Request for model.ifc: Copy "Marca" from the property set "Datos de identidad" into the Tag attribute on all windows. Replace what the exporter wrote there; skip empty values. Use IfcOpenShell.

First a look at what the model holds.

```python
import ifcopenshell
import ifcopenshell.util.element

model = ifcopenshell.open("model.ifc")
print(model.schema)
windows = model.by_type("IfcWindow")
print(len(windows), "windows")
for e in windows[:8]:
    source = ifcopenshell.util.element.get_pset(e, "Datos de identidad", "Marca")
    target = e.Tag
    print(e.id(), repr(source), repr(target), sep=" | ")
```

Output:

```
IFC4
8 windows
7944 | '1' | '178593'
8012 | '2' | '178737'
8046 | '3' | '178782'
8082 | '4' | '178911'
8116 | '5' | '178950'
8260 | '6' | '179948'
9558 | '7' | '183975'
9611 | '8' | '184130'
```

```python
import ifcopenshell
import ifcopenshell.util.element

model = ifcopenshell.open("model.ifc")

count = 0
for e in model.by_type("IfcWindow"):
    value = ifcopenshell.util.element.get_pset(e, "Datos de identidad", "Marca")
    current = e.Tag
    if not value or not value.strip() or current == value:
        continue
    e.Tag = value
    count += 1

print(count, "windows updated")

model.write("model_edited.ifc")
```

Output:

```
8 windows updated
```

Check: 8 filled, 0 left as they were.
